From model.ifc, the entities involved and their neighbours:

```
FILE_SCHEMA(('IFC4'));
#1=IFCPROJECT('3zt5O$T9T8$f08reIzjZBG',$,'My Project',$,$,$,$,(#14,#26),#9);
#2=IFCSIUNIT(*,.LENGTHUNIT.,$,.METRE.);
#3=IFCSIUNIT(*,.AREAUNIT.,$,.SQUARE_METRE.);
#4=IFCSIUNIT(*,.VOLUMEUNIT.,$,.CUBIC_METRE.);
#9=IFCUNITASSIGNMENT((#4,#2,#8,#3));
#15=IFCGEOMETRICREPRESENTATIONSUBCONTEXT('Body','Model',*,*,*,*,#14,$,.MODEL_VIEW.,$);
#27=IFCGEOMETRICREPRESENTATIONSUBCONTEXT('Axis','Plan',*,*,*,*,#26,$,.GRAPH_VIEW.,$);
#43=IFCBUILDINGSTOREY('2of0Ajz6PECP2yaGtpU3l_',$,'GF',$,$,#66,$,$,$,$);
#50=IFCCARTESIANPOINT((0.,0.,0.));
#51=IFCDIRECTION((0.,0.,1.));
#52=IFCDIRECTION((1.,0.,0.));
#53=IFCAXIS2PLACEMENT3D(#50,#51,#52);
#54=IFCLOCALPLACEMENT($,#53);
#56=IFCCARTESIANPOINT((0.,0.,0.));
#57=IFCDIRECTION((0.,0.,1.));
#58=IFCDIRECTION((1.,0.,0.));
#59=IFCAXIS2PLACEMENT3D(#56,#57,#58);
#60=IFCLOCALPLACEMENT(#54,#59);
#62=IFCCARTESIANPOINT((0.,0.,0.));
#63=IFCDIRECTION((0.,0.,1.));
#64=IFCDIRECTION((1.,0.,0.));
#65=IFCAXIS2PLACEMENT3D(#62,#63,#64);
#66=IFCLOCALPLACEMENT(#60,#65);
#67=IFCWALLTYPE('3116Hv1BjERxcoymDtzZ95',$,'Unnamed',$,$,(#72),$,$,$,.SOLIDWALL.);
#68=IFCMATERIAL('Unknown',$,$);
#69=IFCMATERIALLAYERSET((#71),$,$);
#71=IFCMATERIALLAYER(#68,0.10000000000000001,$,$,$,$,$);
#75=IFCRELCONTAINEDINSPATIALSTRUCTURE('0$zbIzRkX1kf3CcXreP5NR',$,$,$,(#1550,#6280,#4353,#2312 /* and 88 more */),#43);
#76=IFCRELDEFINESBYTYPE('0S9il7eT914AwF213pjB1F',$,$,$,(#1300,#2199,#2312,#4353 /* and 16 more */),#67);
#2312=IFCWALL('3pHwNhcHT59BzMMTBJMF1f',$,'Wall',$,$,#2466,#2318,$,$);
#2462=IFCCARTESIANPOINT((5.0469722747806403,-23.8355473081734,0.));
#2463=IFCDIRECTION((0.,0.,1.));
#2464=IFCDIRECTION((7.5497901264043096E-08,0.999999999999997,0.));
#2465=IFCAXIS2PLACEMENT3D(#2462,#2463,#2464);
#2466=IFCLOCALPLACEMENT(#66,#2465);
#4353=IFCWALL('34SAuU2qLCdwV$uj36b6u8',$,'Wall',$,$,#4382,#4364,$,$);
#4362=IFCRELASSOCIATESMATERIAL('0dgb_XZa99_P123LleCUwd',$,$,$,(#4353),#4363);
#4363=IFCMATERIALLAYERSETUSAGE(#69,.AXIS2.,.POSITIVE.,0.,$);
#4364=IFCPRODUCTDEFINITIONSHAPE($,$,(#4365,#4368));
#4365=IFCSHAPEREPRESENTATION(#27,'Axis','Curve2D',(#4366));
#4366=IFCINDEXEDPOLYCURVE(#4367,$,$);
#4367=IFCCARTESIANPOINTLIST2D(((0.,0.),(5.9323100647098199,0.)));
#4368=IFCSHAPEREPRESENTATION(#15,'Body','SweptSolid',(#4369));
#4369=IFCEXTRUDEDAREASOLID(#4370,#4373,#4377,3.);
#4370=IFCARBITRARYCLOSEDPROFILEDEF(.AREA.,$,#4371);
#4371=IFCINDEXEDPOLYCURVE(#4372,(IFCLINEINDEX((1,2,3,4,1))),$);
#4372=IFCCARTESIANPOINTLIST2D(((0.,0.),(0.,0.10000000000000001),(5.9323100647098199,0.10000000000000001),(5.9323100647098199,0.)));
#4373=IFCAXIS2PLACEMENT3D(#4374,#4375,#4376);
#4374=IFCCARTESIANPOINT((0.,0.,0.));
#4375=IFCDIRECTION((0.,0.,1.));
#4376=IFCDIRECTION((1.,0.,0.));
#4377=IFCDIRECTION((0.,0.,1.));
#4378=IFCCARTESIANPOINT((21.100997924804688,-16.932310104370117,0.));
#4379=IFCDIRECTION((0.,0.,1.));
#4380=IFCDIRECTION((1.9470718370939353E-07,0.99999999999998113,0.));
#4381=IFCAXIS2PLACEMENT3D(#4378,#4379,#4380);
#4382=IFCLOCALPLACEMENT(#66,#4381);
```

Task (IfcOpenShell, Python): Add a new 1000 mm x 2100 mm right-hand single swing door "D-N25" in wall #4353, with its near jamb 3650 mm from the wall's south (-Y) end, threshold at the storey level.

```python
import numpy as np
import ifcopenshell
import ifcopenshell.api.feature
import ifcopenshell.api.geometry
import ifcopenshell.api.root
import ifcopenshell.api.spatial
import ifcopenshell.geom
import ifcopenshell.util.element
import ifcopenshell.util.placement
import ifcopenshell.util.representation
import ifcopenshell.util.shape
import ifcopenshell.util.unit

model = ifcopenshell.open("model.ifc")
unit_scale = ifcopenshell.util.unit.calculate_unit_scale(model)
settings = ifcopenshell.geom.settings()


def volume(element):
    """Net volume in cubic metres, openings subtracted."""
    shape = ifcopenshell.geom.create_shape(settings, element)
    return ifcopenshell.util.shape.get_volume(shape.geometry)


wall = model.by_id(4353)
storey = ifcopenshell.util.element.get_container(wall, ifc_class="IfcBuildingStorey")
context = ifcopenshell.util.representation.get_context(model, "Model", "Body", "MODEL_VIEW")
before = volume(wall)

width, height, from_end, sill = 1, 2.1, 3.65, 0.0  # metres

# The wall runs along its own X axis, and the end named is its -X end.
wall_shape = ifcopenshell.geom.create_shape(settings, wall)
x, y, z = ifcopenshell.util.shape.get_vertices(wall_shape.geometry).T
start = x.min() + from_end
face, thickness = float(y.min()), float(y.max() - y.min())
wall_matrix = ifcopenshell.util.placement.get_local_placement(wall.ObjectPlacement)
level = ifcopenshell.util.placement.get_local_placement(storey.ObjectPlacement)[2, 3]


def in_wall(x, y):
    """Placement at x, y metres in the wall's axes, at sill height."""
    matrix = wall_matrix.copy()
    matrix[:, 3] = wall_matrix @ np.array([x / unit_scale, y / unit_scale, 0.0, 1.0])
    matrix[2, 3] = level + sill / unit_scale
    return matrix


# Opening: a box that overshoots both wall faces by 50 mm.
opening = ifcopenshell.api.root.create_entity(model, ifc_class="IfcOpeningElement", predefined_type="OPENING")
box = ifcopenshell.api.geometry.add_wall_representation(
    model, context=context, length=width, height=height, thickness=thickness + 0.1
)
ifcopenshell.api.geometry.assign_representation(model, product=opening, representation=box)
ifcopenshell.api.geometry.edit_object_placement(model, product=opening, matrix=in_wall(start, face - 0.05), is_si=False)
ifcopenshell.api.feature.add_feature(model, feature=opening, element=wall)

door = ifcopenshell.api.root.create_entity(model, ifc_class="IfcDoor", name="D-N25", predefined_type="DOOR")
door.OverallWidth, door.OverallHeight = width / unit_scale, height / unit_scale
door.OperationType = "SINGLE_SWING_RIGHT"
body = ifcopenshell.api.geometry.add_door_representation(
    model,
    context=context,
    overall_width=door.OverallWidth,
    overall_height=door.OverallHeight,
    operation_type="SINGLE_SWING_RIGHT",
    lining_properties={"LiningDepth": thickness / unit_scale, "ThresholdDepth": thickness / unit_scale},
)
ifcopenshell.api.geometry.assign_representation(model, product=door, representation=body)
ifcopenshell.api.spatial.assign_container(model, products=[door], relating_structure=storey)
ifcopenshell.api.feature.add_filling(model, opening=opening, element=door)

# The lining spans the wall, so the door starts at the wall face.
ifcopenshell.api.geometry.edit_object_placement(model, product=door, matrix=in_wall(start, face), is_si=False)

after = volume(wall)

print(f"wall volume {before:.3f} -> {after:.3f} m3")

model.write("model_updated.ifc")
```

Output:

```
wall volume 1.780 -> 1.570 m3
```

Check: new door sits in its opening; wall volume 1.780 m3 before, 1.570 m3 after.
